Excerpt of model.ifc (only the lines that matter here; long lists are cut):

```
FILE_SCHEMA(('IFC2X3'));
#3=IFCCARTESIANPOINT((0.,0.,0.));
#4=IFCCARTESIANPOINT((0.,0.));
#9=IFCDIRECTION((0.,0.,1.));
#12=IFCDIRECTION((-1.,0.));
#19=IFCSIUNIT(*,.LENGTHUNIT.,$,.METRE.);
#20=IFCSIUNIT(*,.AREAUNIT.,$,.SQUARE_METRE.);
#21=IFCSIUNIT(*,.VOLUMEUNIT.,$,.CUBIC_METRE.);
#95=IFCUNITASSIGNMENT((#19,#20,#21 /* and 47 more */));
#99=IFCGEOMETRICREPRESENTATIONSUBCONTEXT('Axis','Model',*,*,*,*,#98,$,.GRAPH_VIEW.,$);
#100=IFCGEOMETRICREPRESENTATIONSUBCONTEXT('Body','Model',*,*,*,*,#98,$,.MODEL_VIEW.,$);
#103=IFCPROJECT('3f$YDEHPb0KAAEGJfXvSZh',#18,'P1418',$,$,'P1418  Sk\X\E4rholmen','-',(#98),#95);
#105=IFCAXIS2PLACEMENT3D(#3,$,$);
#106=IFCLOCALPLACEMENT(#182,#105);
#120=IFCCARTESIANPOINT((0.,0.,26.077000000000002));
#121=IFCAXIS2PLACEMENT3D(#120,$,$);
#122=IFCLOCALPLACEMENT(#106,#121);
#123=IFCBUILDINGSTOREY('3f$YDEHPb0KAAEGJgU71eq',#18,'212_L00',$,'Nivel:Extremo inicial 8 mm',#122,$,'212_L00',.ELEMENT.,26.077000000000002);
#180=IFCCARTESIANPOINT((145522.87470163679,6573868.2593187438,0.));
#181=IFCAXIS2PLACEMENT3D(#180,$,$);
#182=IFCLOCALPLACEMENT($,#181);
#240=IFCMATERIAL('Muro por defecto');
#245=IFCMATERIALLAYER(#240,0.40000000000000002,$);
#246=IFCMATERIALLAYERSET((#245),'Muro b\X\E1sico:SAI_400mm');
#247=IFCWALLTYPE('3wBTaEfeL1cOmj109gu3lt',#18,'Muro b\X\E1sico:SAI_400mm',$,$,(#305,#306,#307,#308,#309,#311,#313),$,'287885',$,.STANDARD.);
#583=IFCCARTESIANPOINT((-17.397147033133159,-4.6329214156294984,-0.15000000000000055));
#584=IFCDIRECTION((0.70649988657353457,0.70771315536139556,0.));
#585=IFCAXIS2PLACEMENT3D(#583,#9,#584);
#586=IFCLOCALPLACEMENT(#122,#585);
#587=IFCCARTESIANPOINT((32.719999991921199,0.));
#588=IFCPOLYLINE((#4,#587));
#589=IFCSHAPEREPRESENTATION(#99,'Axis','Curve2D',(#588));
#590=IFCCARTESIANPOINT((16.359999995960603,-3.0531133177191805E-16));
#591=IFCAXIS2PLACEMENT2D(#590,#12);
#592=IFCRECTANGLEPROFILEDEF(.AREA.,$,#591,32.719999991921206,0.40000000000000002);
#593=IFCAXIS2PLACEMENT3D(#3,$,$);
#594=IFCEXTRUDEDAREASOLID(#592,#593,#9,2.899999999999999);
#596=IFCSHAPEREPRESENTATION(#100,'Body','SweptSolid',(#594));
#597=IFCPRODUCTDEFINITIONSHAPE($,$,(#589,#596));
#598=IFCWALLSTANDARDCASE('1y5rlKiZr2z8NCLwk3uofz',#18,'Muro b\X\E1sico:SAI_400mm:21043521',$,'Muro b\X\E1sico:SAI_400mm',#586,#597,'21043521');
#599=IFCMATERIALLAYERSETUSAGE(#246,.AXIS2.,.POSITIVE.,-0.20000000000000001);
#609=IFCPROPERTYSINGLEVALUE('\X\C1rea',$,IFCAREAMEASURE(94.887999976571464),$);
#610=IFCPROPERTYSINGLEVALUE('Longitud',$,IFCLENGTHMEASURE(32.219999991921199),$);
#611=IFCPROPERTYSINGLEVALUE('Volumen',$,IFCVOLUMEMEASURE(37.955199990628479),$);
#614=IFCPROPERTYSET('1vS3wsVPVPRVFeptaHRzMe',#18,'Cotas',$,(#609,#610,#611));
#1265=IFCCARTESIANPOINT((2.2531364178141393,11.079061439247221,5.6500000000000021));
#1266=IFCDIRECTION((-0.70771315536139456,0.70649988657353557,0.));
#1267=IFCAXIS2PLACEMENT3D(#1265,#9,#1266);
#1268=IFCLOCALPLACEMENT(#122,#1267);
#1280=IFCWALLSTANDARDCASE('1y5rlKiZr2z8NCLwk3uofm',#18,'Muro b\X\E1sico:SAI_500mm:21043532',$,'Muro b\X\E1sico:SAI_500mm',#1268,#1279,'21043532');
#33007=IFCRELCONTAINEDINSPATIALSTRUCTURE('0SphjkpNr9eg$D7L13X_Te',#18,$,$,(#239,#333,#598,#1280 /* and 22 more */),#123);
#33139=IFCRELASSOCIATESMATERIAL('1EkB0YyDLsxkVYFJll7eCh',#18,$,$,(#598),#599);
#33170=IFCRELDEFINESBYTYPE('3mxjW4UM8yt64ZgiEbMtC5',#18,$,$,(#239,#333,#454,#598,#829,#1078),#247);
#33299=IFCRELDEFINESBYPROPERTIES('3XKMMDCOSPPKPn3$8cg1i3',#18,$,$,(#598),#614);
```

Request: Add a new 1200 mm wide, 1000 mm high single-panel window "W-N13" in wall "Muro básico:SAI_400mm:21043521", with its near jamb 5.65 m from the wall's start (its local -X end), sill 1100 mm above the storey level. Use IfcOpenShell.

```python
import numpy as np
import ifcopenshell
import ifcopenshell.api.feature
import ifcopenshell.api.geometry
import ifcopenshell.api.pset
import ifcopenshell.api.root
import ifcopenshell.api.spatial
import ifcopenshell.api.type
import ifcopenshell.geom
import ifcopenshell.util.element
import ifcopenshell.util.placement
import ifcopenshell.util.representation
import ifcopenshell.util.shape
import ifcopenshell.util.unit

model = ifcopenshell.open("model.ifc")
unit_scale = ifcopenshell.util.unit.calculate_unit_scale(model)
area_scale = ifcopenshell.util.unit.calculate_unit_scale(model, "AREAUNIT")
volume_scale = ifcopenshell.util.unit.calculate_unit_scale(model, "VOLUMEUNIT")
settings = ifcopenshell.geom.settings()


def volume(element):
    """Net volume in cubic metres, openings subtracted."""
    shape = ifcopenshell.geom.create_shape(settings, element)
    return ifcopenshell.util.shape.get_volume(shape.geometry)


wall = model.by_guid("1y5rlKiZr2z8NCLwk3uofz")
storey = ifcopenshell.util.element.get_container(wall, ifc_class="IfcBuildingStorey")
context = ifcopenshell.util.representation.get_context(model, "Model", "Body", "MODEL_VIEW")
before = volume(wall)

width, height, from_end, sill = 1.2, 1, 5.65, 1.1  # metres

# The wall runs along its own X axis, and the end named is its -X end.
wall_shape = ifcopenshell.geom.create_shape(settings, wall)
x, y, z = ifcopenshell.util.shape.get_vertices(wall_shape.geometry).T
start = x.min() + from_end
face, thickness = float(y.min()), float(y.max() - y.min())
wall_matrix = ifcopenshell.util.placement.get_local_placement(wall.ObjectPlacement)
level = ifcopenshell.util.placement.get_local_placement(storey.ObjectPlacement)[2, 3]


def in_wall(x, y):
    """Placement at x, y metres in the wall's axes, at sill height."""
    matrix = wall_matrix.copy()
    matrix[:, 3] = wall_matrix @ np.array([x / unit_scale, y / unit_scale, 0.0, 1.0])
    matrix[2, 3] = level + sill / unit_scale
    return matrix


# Opening: a box that overshoots both wall faces by 50 mm.
opening = ifcopenshell.api.root.create_entity(model, ifc_class="IfcOpeningElement")
box = ifcopenshell.api.geometry.add_wall_representation(
    model, context=context, length=width, height=height, thickness=thickness + 0.1
)
ifcopenshell.api.geometry.assign_representation(model, product=opening, representation=box)
ifcopenshell.api.geometry.edit_object_placement(model, product=opening, matrix=in_wall(start, face - 0.05), is_si=False)
ifcopenshell.api.feature.add_feature(model, feature=opening, element=wall)

window = ifcopenshell.api.root.create_entity(model, ifc_class="IfcWindow", name="W-N13")
window.OverallWidth, window.OverallHeight = width / unit_scale, height / unit_scale
body = ifcopenshell.api.geometry.add_window_representation(
    model,
    context=context,
    overall_width=window.OverallWidth,
    overall_height=window.OverallHeight,
    partition_type="SINGLE_PANEL",
)
ifcopenshell.api.geometry.assign_representation(model, product=window, representation=body)
ifcopenshell.api.spatial.assign_container(model, products=[window], relating_structure=storey)
fills = ifcopenshell.api.feature.add_filling(model, opening=opening, element=window)
fills.OwnerHistory = window.OwnerHistory  # required in IFC2X3

# IFC2X3 keeps the operation on the window style.
style = ifcopenshell.api.root.create_entity(model, ifc_class="IfcWindowStyle", name="W-N13")
style.OperationType, style.ConstructionType = "SINGLE_PANEL", "NOTDEFINED"
style.ParameterTakesPrecedence = style.Sizeable = False
ifcopenshell.api.type.assign_type(model, related_objects=[window], relating_type=style)

# Centre the window in the wall's thickness.
ifcopenshell.api.geometry.edit_object_placement(model, product=window, matrix=in_wall(start, face), is_si=False)
window_shape = ifcopenshell.geom.create_shape(settings, window)
depth = ifcopenshell.util.shape.get_vertices(window_shape.geometry)[:, 1]
offset = face + thickness / 2 - (depth.min() + depth.max()) / 2
ifcopenshell.api.geometry.edit_object_placement(model, product=window, matrix=in_wall(start, offset), is_si=False)

after = volume(wall)

# Update the wall's stored quantities.
pset = model.by_id(ifcopenshell.util.element.get_pset(wall, "Cotas", should_inherit=False)["id"])
ifcopenshell.api.pset.edit_pset(model, pset=pset, properties={
    "Área": model.create_entity("IfcAreaMeasure", after / thickness / area_scale),
    "Volumen": model.create_entity("IfcVolumeMeasure", after / volume_scale),
})

print(f"wall volume {before:.3f} -> {after:.3f} m3")

model.write("model_v2.ifc")
```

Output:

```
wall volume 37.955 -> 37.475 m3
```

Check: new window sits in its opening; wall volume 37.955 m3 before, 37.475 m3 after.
